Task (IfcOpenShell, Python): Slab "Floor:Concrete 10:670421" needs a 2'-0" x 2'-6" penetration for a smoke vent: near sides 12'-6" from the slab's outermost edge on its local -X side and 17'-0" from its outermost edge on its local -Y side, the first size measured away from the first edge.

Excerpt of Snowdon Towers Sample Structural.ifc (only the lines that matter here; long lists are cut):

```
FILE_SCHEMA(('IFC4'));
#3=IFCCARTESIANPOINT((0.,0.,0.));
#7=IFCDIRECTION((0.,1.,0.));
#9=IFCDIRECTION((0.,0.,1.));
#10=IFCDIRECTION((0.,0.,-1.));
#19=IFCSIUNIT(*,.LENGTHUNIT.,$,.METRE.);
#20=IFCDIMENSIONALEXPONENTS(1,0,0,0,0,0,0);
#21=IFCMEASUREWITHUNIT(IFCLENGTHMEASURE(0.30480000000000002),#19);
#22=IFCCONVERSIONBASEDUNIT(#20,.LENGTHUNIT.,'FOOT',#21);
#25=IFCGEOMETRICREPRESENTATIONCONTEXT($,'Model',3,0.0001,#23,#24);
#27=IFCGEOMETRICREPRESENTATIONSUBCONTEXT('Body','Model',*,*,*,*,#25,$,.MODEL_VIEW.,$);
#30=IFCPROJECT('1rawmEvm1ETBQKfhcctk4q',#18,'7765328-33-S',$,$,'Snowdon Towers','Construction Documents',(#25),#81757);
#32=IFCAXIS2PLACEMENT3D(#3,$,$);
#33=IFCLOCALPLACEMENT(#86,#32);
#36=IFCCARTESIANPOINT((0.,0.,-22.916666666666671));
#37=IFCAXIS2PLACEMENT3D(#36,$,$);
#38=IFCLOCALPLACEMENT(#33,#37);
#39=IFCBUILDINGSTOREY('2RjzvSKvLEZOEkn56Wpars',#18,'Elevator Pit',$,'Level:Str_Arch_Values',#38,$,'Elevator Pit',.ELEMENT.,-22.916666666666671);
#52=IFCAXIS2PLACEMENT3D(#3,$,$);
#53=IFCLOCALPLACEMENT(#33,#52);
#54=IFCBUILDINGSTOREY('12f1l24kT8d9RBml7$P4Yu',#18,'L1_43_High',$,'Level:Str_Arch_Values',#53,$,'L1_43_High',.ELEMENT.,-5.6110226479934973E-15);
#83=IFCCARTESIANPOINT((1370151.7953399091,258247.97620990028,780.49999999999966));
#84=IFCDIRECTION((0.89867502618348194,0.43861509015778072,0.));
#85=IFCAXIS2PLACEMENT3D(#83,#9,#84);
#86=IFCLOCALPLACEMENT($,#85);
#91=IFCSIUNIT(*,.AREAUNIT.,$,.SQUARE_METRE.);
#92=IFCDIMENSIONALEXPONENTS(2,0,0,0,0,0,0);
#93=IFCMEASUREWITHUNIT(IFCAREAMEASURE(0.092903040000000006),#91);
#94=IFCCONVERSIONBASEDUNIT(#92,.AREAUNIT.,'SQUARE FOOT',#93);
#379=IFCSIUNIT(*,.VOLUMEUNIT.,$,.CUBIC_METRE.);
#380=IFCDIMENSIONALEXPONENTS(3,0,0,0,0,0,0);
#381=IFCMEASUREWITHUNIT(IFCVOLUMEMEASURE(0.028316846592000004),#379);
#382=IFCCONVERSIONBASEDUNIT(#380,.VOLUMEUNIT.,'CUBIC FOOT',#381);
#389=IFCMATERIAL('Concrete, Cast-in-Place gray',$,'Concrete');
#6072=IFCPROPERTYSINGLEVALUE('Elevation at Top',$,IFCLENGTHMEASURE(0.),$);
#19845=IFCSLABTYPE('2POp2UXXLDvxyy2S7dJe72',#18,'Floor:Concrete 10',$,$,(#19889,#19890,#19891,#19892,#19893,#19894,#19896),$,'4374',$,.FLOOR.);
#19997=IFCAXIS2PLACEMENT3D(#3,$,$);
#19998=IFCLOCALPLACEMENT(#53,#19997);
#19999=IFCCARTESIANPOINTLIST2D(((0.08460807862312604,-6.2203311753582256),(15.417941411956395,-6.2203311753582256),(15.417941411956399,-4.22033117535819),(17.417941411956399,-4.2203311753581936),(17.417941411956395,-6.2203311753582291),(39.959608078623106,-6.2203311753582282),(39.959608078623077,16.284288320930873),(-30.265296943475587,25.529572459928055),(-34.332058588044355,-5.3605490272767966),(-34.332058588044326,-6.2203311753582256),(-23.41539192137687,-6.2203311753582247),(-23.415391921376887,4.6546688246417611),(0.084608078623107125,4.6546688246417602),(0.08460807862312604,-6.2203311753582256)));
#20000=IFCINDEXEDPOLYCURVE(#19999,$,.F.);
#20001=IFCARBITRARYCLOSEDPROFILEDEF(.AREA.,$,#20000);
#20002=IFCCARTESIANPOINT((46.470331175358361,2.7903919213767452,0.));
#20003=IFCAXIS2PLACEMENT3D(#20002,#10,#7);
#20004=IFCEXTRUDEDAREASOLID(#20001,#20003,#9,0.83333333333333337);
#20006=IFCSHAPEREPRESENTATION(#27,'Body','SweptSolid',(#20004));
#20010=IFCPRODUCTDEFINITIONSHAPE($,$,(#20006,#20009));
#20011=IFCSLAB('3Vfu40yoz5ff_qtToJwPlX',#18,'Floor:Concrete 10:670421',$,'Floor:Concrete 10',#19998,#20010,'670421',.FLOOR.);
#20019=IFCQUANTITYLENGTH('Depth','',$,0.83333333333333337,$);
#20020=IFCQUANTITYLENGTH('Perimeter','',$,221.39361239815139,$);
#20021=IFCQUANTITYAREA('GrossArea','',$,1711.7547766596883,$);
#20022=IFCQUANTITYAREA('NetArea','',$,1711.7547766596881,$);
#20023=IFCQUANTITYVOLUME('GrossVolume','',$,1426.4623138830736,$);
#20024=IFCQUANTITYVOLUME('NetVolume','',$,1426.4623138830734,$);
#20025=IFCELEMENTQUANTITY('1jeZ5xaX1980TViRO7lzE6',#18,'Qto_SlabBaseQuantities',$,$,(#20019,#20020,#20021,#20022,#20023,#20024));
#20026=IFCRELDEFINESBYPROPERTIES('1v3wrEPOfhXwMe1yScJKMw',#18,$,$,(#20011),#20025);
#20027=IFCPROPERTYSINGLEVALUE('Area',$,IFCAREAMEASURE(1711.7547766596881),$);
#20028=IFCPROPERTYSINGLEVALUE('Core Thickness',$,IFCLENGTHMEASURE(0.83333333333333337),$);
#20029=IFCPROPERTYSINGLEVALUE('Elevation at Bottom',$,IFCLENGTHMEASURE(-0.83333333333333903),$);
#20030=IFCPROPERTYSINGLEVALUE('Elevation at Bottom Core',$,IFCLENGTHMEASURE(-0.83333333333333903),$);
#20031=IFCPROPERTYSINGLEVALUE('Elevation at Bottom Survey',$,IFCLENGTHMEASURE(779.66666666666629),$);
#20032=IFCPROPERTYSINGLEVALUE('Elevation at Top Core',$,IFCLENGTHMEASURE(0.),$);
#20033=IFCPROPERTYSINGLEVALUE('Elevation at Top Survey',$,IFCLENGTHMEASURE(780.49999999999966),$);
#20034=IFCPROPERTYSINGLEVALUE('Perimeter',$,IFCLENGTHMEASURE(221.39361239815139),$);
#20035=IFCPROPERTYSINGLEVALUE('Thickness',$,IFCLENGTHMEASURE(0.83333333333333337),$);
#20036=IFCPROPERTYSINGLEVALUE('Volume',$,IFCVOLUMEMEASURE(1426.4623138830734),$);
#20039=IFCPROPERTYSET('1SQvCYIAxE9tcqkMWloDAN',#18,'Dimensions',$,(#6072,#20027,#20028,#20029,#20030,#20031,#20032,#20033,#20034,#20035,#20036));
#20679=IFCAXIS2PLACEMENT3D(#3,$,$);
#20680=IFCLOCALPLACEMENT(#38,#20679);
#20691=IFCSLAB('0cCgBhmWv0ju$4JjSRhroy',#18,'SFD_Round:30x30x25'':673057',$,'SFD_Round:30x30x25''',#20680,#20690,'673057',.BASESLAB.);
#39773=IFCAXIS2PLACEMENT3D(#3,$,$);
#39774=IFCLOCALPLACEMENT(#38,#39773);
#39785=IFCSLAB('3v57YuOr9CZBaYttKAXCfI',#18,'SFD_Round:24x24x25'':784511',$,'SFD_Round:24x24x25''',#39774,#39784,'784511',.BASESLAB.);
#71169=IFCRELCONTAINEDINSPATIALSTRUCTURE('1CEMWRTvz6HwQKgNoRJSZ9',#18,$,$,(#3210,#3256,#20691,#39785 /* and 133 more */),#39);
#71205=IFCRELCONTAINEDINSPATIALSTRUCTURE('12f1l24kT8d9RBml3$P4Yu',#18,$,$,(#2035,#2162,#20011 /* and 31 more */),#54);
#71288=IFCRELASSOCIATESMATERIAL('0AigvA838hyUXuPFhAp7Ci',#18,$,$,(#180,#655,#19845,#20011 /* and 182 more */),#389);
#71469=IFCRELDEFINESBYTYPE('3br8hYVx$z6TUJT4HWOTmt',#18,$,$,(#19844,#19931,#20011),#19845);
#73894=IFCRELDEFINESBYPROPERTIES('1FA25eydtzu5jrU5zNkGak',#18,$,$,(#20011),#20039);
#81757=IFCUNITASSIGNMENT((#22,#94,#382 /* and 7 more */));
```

```python
import numpy as np
import ifcopenshell
import ifcopenshell.api.feature
import ifcopenshell.api.geometry
import ifcopenshell.api.pset
import ifcopenshell.api.root
import ifcopenshell.geom
import ifcopenshell.util.element
import ifcopenshell.util.placement
import ifcopenshell.util.representation
import ifcopenshell.util.shape
import ifcopenshell.util.unit

model = ifcopenshell.open("Snowdon Towers Sample Structural.ifc")
unit_scale = ifcopenshell.util.unit.calculate_unit_scale(model)
area_scale = ifcopenshell.util.unit.calculate_unit_scale(model, "AREAUNIT")
volume_scale = ifcopenshell.util.unit.calculate_unit_scale(model, "VOLUMEUNIT")
settings = ifcopenshell.geom.settings()


def volume(element):
    """Net volume in cubic metres, openings subtracted."""
    shape = ifcopenshell.geom.create_shape(settings, element)
    return ifcopenshell.util.shape.get_volume(shape.geometry)


slab = model.by_guid("3Vfu40yoz5ff_qtToJwPlX")
before = volume(slab)

# Extent in the slab's own axes, in metres. The edges named are its -X and -Y sides.
slab_shape = ifcopenshell.geom.create_shape(settings, slab)
vertices = ifcopenshell.util.shape.get_vertices(slab_shape.geometry)
x_min, y_min, bottom = vertices.min(axis=0)
top = vertices[:, 2].max()

opening = ifcopenshell.api.root.create_entity(model, ifc_class="IfcOpeningElement", name="Smoke vent opening", predefined_type="OPENING")
context = ifcopenshell.util.representation.get_context(model, "Model", "Body", "MODEL_VIEW")
width, depth = 0.6096, 0.762
outline = [(0.0, 0.0), (width, 0.0), (width, depth), (0.0, depth), (0.0, 0.0)]
# Overshoot both faces by 50 mm so the cut is clean.
shape = ifcopenshell.api.geometry.add_slab_representation(
    model, context=context, depth=top - bottom + 0.1, polyline=outline
)
ifcopenshell.api.geometry.assign_representation(model, product=opening, representation=shape)

matrix = ifcopenshell.util.placement.get_local_placement(slab.ObjectPlacement)
matrix[:, 3] = matrix @ np.append(np.array([x_min + 3.81, y_min + 5.1816, bottom - 0.05]) / unit_scale, 1.0)
ifcopenshell.api.geometry.edit_object_placement(model, product=opening, matrix=matrix, is_si=False)
ifcopenshell.api.feature.add_feature(model, feature=opening, element=slab)

after = volume(slab)

# Update the slab's stored quantities.
qto = model.by_id(ifcopenshell.util.element.get_pset(slab, "Qto_SlabBaseQuantities", should_inherit=False)["id"])
ifcopenshell.api.pset.edit_qto(model, qto=qto, properties={
    "NetArea": after / (top - bottom) / area_scale,
    "NetVolume": after / volume_scale,
})
pset = model.by_id(ifcopenshell.util.element.get_pset(slab, "Dimensions", should_inherit=False)["id"])
ifcopenshell.api.pset.edit_pset(model, pset=pset, properties={
    "Area": model.create_entity("IfcAreaMeasure", after / (top - bottom) / area_scale),
    "Volume": model.create_entity("IfcVolumeMeasure", after / volume_scale),
})

print(f"slab volume {before:.3f} -> {after:.3f} m3")

model.write("Snowdon Towers Sample Structural_updated.ifc")
```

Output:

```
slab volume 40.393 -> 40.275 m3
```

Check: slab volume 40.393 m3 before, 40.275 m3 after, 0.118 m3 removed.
